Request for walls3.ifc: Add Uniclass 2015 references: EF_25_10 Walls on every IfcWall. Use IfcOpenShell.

First a look at what the model holds.

```python
import ifcopenshell

model = ifcopenshell.open("walls3.ifc")
print(model.schema)
print("classifications:", [c.Name for c in model.by_type("IfcClassification")])
for ifc_class in ("IfcDoor", "IfcRoof", "IfcStair", "IfcWall", "IfcWindow"):
    print(ifc_class, len(model.by_type(ifc_class)))
```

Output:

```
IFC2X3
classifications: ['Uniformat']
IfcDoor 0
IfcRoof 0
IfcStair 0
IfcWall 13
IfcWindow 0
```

```python
import ifcopenshell
import ifcopenshell.api.classification

model = ifcopenshell.open("walls3.ifc")

# IFC2X3 requires Source and Edition and has no link from the project to the system.
system = model.create_entity("IfcClassification", Source="NBS", Edition="2015", Name="Uniclass 2015")

codes = {
    "IfcWall": ("EF_25_10", "Walls"),
}
for ifc_class, (code, name) in codes.items():
    products = model.by_type(ifc_class)
    ifcopenshell.api.classification.add_reference(
        model, products=products, classification=system, identification=code, name=name
    )
    print(code, len(products))

model.write("walls3_rev.ifc")
```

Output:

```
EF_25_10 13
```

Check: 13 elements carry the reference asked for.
